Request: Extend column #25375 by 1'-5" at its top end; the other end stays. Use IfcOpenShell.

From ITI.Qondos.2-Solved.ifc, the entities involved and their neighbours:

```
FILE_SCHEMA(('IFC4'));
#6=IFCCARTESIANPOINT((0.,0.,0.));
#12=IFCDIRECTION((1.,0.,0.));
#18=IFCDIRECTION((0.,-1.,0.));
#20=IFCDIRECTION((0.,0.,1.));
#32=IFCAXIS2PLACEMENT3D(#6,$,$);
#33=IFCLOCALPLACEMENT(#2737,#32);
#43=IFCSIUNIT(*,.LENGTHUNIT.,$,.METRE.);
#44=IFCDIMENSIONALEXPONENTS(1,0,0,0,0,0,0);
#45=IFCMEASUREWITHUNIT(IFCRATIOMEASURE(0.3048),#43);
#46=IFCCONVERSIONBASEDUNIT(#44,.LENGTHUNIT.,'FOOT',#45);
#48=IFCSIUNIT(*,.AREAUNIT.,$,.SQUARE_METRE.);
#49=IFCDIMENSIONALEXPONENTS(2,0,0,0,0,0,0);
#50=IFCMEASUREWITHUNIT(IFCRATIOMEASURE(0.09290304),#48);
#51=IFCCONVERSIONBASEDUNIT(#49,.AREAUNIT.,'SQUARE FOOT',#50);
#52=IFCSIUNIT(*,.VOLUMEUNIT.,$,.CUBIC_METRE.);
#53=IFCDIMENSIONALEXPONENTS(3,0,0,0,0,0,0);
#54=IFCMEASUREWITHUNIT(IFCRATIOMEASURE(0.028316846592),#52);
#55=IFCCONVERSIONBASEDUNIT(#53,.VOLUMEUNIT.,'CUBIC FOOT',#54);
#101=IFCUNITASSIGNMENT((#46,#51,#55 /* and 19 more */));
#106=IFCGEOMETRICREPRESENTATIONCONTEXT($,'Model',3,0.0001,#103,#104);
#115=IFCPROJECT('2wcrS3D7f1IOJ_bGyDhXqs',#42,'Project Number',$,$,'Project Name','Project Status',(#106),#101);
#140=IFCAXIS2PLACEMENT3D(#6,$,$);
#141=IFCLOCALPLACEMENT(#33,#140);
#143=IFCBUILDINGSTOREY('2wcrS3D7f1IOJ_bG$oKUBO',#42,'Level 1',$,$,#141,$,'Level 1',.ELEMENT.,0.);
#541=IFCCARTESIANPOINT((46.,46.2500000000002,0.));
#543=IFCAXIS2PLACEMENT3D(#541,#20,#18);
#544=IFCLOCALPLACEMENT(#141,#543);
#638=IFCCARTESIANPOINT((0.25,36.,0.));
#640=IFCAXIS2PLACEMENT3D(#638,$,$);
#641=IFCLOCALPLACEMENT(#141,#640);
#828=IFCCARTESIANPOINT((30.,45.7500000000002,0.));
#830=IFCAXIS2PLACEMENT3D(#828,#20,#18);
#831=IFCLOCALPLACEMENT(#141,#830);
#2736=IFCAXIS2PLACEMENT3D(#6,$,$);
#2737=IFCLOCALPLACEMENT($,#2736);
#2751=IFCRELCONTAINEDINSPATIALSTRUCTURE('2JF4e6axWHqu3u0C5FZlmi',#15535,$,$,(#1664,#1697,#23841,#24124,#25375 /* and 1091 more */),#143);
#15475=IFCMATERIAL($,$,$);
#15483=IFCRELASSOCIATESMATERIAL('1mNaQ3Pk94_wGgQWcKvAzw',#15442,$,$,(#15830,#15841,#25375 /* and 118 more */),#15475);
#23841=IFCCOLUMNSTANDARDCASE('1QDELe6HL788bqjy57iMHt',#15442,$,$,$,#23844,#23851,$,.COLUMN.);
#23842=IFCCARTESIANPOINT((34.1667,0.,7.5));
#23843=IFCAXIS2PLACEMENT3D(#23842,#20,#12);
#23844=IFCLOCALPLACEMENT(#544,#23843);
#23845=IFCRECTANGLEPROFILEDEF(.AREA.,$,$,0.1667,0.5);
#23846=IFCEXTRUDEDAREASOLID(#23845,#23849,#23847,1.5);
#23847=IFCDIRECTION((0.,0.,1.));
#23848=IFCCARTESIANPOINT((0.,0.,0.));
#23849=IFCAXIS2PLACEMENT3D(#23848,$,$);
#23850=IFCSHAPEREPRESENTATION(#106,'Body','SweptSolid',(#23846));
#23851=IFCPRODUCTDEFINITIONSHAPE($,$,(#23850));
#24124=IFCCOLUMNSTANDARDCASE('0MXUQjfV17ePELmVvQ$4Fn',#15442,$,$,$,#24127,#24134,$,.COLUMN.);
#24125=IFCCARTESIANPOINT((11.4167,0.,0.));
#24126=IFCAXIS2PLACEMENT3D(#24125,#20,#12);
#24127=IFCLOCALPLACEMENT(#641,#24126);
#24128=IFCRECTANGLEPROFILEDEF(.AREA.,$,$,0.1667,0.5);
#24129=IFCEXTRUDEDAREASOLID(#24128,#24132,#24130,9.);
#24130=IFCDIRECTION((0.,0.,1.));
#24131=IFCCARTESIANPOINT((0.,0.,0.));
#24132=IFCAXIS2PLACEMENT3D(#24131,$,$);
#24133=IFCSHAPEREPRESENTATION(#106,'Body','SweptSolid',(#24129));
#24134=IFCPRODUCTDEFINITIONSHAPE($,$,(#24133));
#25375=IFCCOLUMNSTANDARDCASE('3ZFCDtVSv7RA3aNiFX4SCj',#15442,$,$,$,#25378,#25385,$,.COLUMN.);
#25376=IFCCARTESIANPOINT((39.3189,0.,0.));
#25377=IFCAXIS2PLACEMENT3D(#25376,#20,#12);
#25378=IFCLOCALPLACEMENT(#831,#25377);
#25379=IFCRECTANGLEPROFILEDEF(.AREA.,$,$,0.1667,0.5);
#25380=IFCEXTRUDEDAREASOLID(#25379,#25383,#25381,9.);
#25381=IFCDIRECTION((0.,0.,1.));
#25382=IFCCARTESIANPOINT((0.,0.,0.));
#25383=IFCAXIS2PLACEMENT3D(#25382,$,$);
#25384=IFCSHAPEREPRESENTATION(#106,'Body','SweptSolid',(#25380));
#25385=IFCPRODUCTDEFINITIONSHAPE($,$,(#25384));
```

```python
import ifcopenshell
import ifcopenshell.util.unit

model = ifcopenshell.open("ITI.Qondos.2-Solved.ifc")
unit_scale = ifcopenshell.util.unit.calculate_unit_scale(model)

member = model.by_guid("3ZFCDtVSv7RA3aNiFX4SCj")
change = 17 * 0.0254 / unit_scale

# The extrusion runs towards the end named, so only its depth changes.
body = next(r for r in member.Representation.Representations if r.RepresentationIdentifier == "Body")
solid = body.Items[0]
old_length = solid.Depth
solid.Depth += change

print(f"length {old_length:g} -> {solid.Depth:g}")

model.write("ITI.Qondos.2-Solved-out.ifc")
```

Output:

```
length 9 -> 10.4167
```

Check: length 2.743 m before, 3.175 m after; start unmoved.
